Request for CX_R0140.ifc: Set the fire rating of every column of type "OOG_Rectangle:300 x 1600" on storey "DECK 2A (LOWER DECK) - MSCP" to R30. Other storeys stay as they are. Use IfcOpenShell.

First a look at what the model holds.

```python
import ifcopenshell
import ifcopenshell.util.element

model = ifcopenshell.open("CX_R0140.ifc")
print(model.schema)
storey = next(s for s in model.by_type("IfcBuildingStorey") if s.Name == "DECK 2A (LOWER DECK) - MSCP")
columns = [e for e in ifcopenshell.util.element.get_decomposition(storey) if e.is_a("IfcColumn")]
seen = {}
for e in columns:
    element_type = ifcopenshell.util.element.get_type(e)
    key = (element_type.Name if element_type != e and element_type else None, ifcopenshell.util.element.get_pset(e, "Pset_ColumnCommon", "FireRating"))
    seen[key] = seen.get(key, 0) + 1
for (name, value), count in sorted(seen.items(), key=str):
    print(count, "x", name, "|", value)
```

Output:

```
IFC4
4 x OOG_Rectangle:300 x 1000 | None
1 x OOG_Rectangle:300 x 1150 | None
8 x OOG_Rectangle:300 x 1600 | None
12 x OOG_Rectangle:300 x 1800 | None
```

```python
import ifcopenshell
import ifcopenshell.api.pset
import ifcopenshell.util.element

model = ifcopenshell.open("CX_R0140.ifc")

storey = next(s for s in model.by_type("IfcBuildingStorey") if s.Name == "DECK 2A (LOWER DECK) - MSCP")
columns = [e for e in ifcopenshell.util.element.get_decomposition(storey) if e.is_a("IfcColumn")]

count = 0
for e in columns:
    element_type = ifcopenshell.util.element.get_type(e)
    if element_type in (None, e) or element_type.Name != "OOG_Rectangle:300 x 1600":
        continue
    # add_pset returns the element's existing set when there is one.
    pset = ifcopenshell.api.pset.add_pset(model, product=e, name="Pset_ColumnCommon")
    ifcopenshell.api.pset.edit_pset(model, pset=pset, properties={"FireRating": "R30"})
    count += 1

print(count, "columns updated")

model.write("CX_R0140_edited.ifc")
```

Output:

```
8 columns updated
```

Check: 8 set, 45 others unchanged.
